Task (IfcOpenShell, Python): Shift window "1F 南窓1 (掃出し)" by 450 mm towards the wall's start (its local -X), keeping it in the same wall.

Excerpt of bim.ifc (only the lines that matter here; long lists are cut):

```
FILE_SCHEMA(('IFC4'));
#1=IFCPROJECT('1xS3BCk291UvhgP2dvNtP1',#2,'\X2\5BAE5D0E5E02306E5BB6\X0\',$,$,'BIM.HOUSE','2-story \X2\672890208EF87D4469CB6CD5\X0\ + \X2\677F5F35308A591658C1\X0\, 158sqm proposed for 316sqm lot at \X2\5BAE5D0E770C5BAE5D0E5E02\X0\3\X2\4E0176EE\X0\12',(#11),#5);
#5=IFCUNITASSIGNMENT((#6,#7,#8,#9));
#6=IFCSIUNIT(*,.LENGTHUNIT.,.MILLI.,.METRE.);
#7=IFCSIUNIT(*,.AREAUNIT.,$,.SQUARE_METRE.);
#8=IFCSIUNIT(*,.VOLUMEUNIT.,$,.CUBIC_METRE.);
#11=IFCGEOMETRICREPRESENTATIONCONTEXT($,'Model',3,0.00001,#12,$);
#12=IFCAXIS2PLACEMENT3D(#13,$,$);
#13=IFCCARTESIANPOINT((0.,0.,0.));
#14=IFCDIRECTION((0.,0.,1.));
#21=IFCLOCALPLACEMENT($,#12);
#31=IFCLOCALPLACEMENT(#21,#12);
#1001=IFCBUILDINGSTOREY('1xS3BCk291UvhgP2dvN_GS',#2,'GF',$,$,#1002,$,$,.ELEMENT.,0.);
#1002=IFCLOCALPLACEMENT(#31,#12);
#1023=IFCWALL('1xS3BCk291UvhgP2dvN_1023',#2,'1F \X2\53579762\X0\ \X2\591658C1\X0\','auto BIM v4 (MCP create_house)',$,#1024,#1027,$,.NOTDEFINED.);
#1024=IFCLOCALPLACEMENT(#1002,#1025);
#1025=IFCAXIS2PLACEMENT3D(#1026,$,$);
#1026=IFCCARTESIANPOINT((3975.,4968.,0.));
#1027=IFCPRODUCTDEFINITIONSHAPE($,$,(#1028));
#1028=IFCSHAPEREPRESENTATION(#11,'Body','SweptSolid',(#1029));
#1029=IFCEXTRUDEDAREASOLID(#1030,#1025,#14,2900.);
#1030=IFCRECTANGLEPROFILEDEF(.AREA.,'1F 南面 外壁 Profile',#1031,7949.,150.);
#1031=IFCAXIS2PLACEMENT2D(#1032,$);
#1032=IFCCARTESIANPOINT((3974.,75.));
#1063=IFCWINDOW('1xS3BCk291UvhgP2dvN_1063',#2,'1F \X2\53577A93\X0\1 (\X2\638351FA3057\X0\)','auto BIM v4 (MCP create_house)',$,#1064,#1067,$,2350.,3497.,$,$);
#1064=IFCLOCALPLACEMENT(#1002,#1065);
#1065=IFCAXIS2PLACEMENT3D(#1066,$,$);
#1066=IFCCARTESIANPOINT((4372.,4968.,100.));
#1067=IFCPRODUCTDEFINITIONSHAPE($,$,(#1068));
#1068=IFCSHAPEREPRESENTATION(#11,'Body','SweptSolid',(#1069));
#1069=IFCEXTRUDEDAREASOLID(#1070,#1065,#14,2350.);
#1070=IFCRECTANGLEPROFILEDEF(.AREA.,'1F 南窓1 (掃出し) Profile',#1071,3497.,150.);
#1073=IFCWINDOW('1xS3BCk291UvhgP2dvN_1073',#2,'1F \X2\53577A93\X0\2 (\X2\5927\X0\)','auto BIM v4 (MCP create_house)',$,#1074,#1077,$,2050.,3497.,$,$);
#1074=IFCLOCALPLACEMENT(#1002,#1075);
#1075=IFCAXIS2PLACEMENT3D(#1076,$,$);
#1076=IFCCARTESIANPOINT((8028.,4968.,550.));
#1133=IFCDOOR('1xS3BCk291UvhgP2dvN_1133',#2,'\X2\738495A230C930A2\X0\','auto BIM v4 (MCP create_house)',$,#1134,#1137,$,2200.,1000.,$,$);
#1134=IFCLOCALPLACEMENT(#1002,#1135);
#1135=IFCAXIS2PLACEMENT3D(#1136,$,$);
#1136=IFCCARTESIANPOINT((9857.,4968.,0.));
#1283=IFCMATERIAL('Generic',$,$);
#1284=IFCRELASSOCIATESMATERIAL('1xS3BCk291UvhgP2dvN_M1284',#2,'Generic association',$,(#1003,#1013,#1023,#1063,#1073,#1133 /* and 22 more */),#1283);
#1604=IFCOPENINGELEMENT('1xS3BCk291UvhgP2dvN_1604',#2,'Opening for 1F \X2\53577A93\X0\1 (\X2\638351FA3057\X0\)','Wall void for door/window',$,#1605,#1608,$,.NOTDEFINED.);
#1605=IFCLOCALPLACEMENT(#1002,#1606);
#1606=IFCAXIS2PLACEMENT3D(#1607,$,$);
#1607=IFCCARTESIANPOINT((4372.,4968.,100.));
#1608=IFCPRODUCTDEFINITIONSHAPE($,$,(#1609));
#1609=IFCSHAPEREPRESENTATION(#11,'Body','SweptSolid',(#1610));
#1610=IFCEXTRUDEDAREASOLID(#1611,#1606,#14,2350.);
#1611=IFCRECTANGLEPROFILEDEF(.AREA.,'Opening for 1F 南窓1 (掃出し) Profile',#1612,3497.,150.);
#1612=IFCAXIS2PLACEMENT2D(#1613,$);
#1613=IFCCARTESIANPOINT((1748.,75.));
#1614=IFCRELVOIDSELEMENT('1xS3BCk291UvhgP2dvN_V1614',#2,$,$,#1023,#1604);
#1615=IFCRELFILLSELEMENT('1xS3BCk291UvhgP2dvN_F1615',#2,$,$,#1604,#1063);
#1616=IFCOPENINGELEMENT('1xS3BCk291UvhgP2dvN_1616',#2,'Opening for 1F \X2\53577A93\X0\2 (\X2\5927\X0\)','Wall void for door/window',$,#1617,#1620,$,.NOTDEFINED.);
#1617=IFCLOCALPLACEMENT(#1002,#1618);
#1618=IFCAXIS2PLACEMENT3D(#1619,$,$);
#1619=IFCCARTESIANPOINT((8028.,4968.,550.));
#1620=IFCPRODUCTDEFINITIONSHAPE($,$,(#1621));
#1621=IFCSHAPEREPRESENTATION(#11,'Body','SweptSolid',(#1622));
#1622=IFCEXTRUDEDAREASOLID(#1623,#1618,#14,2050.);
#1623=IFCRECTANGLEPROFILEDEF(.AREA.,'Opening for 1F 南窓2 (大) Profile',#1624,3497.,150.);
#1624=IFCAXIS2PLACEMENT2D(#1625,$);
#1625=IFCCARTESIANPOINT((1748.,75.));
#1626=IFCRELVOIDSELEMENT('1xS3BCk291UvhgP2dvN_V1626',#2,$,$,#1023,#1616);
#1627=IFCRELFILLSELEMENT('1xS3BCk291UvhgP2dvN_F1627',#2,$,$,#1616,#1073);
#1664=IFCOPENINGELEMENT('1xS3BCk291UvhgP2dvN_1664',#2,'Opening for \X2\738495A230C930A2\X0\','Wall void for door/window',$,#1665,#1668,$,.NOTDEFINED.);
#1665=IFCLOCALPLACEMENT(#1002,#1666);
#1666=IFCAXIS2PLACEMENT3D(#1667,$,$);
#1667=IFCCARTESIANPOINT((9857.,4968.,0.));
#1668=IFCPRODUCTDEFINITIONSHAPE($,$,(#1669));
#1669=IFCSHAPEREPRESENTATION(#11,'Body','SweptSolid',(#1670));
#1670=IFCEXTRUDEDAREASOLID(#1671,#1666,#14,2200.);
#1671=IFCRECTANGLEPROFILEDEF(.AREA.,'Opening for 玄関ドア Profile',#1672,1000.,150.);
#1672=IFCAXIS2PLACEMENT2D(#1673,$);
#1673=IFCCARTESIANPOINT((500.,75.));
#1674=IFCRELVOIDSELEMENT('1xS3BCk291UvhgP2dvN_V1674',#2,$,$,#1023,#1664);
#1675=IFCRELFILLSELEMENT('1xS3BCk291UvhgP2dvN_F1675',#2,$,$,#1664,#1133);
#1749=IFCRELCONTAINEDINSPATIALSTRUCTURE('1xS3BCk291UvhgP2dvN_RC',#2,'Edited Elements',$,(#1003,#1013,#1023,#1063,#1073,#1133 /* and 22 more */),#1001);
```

```python
import ifcopenshell
import ifcopenshell.api.geometry
import ifcopenshell.util.placement
import ifcopenshell.util.unit

model = ifcopenshell.open("bim.ifc")
unit_scale = ifcopenshell.util.unit.calculate_unit_scale(model)

window = model.by_id(1063)
opening = window.FillsVoids[0].RelatingOpeningElement
wall = opening.VoidsElements[0].RelatingBuildingElement

wall_matrix = ifcopenshell.util.placement.get_local_placement(wall.ObjectPlacement)
shift = wall_matrix[:3, 0] * -0.45 / unit_scale
before = ifcopenshell.util.placement.get_local_placement(window.ObjectPlacement)[:3, 3].copy()

# The window is not placed relative to its opening, so move both.
for product in (opening, window):
    matrix = ifcopenshell.util.placement.get_local_placement(product.ObjectPlacement)
    matrix[:3, 3] += shift
    ifcopenshell.api.geometry.edit_object_placement(model, product=product, matrix=matrix, is_si=False)

after = ifcopenshell.util.placement.get_local_placement(window.ObjectPlacement)[:3, 3]
print("window moved by", (after - before).round(3) + 0.0)

model.write("bim-out.ifc")
```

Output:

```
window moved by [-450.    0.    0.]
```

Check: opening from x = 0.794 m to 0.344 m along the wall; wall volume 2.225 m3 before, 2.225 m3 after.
